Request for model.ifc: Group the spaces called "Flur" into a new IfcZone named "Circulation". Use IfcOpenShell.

First a look at what the model holds.

```python
import ifcopenshell

model = ifcopenshell.open("model.ifc")
print(model.schema)
seen = {}
for space in model.by_type("IfcSpace"):
    seen[space.LongName] = seen.get(space.LongName, 0) + 1
for name, count in sorted(seen.items(), key=str):
    print(count, "x", name)
print("zones:", [z.Name for z in model.by_type("IfcZone")][:20])
```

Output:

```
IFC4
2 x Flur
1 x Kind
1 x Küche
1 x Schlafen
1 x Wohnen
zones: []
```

```python
import ifcopenshell
import ifcopenshell.api.group
import ifcopenshell.api.root

model = ifcopenshell.open("model.ifc")

names = {"Flur"}
spaces = [s for s in model.by_type("IfcSpace") if s.LongName in names]

zone = ifcopenshell.api.root.create_entity(model, ifc_class="IfcZone", name="Circulation")
ifcopenshell.api.group.assign_group(model, products=spaces, group=zone)
print(len(spaces), "spaces in", zone.Name)

model.write("model_updated.ifc")
```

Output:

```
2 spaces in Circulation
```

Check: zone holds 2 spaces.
